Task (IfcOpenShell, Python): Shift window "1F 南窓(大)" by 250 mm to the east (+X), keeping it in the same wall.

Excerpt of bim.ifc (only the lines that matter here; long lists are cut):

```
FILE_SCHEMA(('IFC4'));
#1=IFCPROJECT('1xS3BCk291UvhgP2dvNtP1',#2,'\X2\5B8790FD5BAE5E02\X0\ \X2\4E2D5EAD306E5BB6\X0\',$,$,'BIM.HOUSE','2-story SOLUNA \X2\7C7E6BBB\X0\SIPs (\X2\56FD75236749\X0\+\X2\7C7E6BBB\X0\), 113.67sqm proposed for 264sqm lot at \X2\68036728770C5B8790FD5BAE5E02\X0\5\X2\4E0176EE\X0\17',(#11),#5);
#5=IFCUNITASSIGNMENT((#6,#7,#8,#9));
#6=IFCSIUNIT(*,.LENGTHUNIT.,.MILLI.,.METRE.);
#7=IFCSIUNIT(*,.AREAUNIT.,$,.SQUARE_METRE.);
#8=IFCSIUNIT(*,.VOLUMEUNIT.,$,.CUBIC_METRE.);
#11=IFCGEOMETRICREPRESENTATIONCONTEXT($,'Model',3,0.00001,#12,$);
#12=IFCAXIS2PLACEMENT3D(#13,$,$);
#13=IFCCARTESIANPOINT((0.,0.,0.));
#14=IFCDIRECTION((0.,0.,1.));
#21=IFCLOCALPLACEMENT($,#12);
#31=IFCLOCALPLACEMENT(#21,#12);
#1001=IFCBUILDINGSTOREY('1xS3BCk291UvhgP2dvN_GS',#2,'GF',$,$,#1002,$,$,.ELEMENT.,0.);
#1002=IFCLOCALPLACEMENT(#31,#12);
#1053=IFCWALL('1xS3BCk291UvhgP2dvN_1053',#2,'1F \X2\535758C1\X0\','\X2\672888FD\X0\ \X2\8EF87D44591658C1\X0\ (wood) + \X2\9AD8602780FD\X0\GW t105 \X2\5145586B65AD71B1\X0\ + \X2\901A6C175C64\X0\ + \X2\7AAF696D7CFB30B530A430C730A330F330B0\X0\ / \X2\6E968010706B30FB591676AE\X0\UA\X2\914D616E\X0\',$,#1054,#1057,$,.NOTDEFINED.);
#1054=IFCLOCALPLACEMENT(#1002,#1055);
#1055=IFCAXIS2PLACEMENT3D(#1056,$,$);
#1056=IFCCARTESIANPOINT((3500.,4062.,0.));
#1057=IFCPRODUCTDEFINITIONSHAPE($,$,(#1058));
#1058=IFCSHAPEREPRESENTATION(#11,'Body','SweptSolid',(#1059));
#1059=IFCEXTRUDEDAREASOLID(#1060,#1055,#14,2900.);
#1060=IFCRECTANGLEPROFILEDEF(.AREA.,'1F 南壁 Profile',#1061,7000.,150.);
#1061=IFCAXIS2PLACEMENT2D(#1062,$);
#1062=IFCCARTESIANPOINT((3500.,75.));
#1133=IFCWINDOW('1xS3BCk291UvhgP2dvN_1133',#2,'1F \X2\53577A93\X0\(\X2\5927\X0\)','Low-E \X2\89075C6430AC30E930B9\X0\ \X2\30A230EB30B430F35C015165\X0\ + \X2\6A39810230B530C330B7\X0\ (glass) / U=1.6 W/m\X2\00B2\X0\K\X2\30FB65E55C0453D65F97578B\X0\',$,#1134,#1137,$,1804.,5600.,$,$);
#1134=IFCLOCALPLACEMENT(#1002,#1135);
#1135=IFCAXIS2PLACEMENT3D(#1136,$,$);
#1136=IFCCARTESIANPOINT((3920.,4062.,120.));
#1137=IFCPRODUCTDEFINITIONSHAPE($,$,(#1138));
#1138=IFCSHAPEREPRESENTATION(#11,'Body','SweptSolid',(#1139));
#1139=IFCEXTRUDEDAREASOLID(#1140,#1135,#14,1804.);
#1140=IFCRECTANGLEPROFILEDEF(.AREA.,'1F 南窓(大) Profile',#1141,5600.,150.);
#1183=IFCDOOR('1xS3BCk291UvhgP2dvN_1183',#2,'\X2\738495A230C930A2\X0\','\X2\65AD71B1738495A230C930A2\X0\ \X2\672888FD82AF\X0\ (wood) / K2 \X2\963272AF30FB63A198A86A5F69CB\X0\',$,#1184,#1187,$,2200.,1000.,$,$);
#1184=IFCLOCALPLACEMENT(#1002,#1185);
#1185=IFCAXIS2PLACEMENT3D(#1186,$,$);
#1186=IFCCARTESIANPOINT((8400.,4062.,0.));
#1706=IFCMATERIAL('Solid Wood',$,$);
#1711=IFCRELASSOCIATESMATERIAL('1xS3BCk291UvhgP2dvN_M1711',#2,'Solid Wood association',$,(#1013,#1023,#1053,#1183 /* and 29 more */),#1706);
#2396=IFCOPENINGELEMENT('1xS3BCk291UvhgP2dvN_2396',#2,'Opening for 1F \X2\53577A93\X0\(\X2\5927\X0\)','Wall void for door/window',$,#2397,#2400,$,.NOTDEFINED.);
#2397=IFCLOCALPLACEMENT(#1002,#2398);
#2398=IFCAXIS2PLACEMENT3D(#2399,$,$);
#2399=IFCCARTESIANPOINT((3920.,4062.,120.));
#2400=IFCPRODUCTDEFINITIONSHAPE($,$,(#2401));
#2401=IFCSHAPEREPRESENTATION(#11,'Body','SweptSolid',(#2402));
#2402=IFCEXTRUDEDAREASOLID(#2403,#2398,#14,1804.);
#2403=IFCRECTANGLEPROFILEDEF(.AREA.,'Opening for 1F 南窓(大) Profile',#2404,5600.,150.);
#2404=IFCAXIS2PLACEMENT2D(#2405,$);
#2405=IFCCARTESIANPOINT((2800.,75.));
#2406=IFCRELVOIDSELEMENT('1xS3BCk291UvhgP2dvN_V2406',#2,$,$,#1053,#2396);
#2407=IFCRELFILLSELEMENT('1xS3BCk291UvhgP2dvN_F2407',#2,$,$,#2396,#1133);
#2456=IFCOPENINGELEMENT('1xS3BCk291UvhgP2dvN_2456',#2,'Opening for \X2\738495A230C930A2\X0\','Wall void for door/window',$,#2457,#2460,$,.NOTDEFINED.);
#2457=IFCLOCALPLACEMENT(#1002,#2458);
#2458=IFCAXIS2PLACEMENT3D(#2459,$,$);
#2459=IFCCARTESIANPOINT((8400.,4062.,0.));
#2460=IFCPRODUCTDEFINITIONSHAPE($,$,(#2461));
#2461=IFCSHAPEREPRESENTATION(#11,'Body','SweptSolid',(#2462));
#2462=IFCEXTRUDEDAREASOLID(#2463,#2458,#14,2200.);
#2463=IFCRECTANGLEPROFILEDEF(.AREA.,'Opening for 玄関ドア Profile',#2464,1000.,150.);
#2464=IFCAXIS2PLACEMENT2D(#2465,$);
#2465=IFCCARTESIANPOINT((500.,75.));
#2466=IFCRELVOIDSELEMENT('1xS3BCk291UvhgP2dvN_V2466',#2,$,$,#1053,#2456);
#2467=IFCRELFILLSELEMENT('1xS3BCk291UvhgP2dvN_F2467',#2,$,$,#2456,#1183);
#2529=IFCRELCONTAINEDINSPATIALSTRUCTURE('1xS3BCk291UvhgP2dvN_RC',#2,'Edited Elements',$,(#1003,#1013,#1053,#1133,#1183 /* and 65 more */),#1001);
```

```python
import ifcopenshell
import ifcopenshell.api.geometry
import ifcopenshell.util.placement

model = ifcopenshell.open("bim.ifc")

window = model.by_guid("1xS3BCk291UvhgP2dvN_1133")
opening = window.FillsVoids[0].RelatingOpeningElement
wall = opening.VoidsElements[0].RelatingBuildingElement

wall_matrix = ifcopenshell.util.placement.get_local_placement(wall.ObjectPlacement)
shift = wall_matrix[:3, 0] * 250.0
before = ifcopenshell.util.placement.get_local_placement(window.ObjectPlacement)[:3, 3].copy()

# The window is not placed relative to its opening, so move both.
for product in (opening, window):
    matrix = ifcopenshell.util.placement.get_local_placement(product.ObjectPlacement)
    matrix[:3, 3] += shift
    ifcopenshell.api.geometry.edit_object_placement(model, product=product, matrix=matrix, is_si=False)

after = ifcopenshell.util.placement.get_local_placement(window.ObjectPlacement)[:3, 3]
print("window moved by", (after - before).round(3) + 0.0)

model.write("bim_rev.ifc")
```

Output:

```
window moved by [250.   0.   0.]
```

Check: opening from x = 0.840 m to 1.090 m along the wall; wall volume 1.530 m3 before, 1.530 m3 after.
